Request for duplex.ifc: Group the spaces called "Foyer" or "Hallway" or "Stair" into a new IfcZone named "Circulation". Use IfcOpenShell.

First a look at what the model holds.

```python
import ifcopenshell

model = ifcopenshell.open("duplex.ifc")
print(model.schema)
seen = {}
for space in model.by_type("IfcSpace"):
    seen[space.LongName] = seen.get(space.LongName, 0) + 1
for name, count in sorted(seen.items(), key=str):
    print(count, "x", name)
print("zones:", [z.Name for z in model.by_type("IfcZone")][:20])
```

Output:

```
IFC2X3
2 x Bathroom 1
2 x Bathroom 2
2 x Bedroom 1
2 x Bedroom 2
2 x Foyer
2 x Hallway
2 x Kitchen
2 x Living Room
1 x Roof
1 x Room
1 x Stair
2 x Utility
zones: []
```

```python
import ifcopenshell
import ifcopenshell.api.group
import ifcopenshell.api.root

model = ifcopenshell.open("duplex.ifc")

names = {"Foyer", "Hallway", "Stair"}
spaces = [s for s in model.by_type("IfcSpace") if s.LongName in names]

zone = ifcopenshell.api.root.create_entity(model, ifc_class="IfcZone", name="Circulation")
ifcopenshell.api.group.assign_group(model, products=spaces, group=zone)
print(len(spaces), "spaces in", zone.Name)

model.write("duplex_updated.ifc")
```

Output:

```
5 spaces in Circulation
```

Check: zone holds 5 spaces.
